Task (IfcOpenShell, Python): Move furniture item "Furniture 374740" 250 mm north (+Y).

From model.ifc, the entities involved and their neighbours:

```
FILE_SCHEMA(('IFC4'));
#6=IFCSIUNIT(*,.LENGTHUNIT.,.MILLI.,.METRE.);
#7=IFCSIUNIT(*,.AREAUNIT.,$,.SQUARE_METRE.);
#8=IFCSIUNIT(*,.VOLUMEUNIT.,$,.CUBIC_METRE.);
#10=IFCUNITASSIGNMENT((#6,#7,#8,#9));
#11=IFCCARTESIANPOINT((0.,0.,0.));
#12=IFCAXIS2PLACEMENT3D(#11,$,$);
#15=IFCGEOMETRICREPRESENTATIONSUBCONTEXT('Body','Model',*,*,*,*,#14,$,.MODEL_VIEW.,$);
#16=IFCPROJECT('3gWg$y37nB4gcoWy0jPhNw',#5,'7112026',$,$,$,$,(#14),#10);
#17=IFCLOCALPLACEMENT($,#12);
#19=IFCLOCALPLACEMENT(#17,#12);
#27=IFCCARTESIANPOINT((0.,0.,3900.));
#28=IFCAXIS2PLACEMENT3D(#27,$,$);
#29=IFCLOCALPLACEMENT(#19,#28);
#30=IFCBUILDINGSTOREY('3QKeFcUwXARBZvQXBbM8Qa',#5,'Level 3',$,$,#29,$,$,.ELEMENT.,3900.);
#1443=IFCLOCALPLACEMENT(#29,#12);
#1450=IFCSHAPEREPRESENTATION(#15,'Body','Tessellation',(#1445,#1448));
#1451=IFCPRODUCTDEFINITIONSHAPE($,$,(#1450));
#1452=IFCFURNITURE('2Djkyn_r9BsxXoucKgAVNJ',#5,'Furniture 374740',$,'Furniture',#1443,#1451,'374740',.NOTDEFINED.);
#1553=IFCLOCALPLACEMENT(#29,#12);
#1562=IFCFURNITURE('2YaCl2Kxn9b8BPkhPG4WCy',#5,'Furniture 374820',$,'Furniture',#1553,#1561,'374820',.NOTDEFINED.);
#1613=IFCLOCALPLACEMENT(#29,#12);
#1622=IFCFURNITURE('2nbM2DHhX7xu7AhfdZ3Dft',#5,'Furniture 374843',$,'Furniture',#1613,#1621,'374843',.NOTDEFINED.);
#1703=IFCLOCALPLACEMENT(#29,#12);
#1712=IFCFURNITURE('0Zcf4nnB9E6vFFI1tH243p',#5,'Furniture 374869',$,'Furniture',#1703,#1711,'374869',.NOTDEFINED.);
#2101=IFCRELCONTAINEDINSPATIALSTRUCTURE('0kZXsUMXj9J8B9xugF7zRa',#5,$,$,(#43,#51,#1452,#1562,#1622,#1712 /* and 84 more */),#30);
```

```python
import ifcopenshell
import ifcopenshell.api.geometry
import ifcopenshell.util.placement
import ifcopenshell.util.unit

model = ifcopenshell.open("model.ifc")
unit_scale = ifcopenshell.util.unit.calculate_unit_scale(model)

item = model.by_guid("2Djkyn_r9BsxXoucKgAVNJ")
matrix = ifcopenshell.util.placement.get_local_placement(item.ObjectPlacement)
matrix[1, 3] += 0.25 / unit_scale
ifcopenshell.api.geometry.edit_object_placement(model, product=item, matrix=matrix, is_si=False)

print(ifcopenshell.util.placement.get_local_placement(item.ObjectPlacement).round(3) + 0.0)

model.write("model_updated.ifc")
```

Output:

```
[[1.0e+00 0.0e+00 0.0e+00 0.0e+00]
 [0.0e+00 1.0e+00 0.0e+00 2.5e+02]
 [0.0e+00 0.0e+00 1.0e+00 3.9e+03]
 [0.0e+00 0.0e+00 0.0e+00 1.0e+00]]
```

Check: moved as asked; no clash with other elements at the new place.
